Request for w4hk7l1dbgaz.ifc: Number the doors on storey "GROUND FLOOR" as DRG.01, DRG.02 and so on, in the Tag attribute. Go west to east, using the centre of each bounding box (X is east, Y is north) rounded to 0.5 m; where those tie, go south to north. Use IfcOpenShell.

First a look at what the model holds.

```python
import ifcopenshell
import ifcopenshell.util.element
import ifcopenshell.util.placement

model = ifcopenshell.open("w4hk7l1dbgaz.ifc")
print(model.schema)
storey = next(s for s in model.by_type("IfcBuildingStorey") if s.Name == "GROUND FLOOR")
doors = [e for e in ifcopenshell.util.element.get_decomposition(storey) if e.is_a("IfcDoor")]
for e in sorted(doors, key=lambda e: e.id()):
    origin = ifcopenshell.util.placement.get_local_placement(e.ObjectPlacement)[:3, 3]
    print(e.id(), e.Tag, e.Name, origin.round(2) + 0.0, sep=" | ")
```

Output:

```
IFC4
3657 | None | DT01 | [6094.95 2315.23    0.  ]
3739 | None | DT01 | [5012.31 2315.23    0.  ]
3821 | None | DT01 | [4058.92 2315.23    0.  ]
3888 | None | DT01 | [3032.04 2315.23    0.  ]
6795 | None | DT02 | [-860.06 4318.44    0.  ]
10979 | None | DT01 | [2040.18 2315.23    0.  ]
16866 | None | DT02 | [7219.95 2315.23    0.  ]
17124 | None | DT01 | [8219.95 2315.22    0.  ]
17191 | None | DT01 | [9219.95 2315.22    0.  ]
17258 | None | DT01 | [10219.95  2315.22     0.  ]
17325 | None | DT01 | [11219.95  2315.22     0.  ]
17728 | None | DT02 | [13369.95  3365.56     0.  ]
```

```python
import ifcopenshell
import ifcopenshell.geom
import ifcopenshell.util.element
import ifcopenshell.util.shape

model = ifcopenshell.open("w4hk7l1dbgaz.ifc")
settings = ifcopenshell.geom.settings()
settings.set("use-world-coords", True)


def centre(element):
    shape = ifcopenshell.geom.create_shape(settings, element)
    return ifcopenshell.util.shape.get_bbox_centroid(shape.geometry)


storey = next(s for s in model.by_type("IfcBuildingStorey") if s.Name == "GROUND FLOOR")
doors = [e for e in ifcopenshell.util.element.get_decomposition(storey) if e.is_a("IfcDoor")]

# Insertion points can sit at a corner or the storey origin, so sort by the geometry (in metres).
centres = {e: centre(e) for e in doors}
doors.sort(key=lambda e: (round(centres[e][0] / 0.5), centres[e][1]))

for i, e in enumerate(doors, start=1):
    number = f"DRG.{i:02d}"
    e.Tag = number
    print(e.id(), number)

model.write("w4hk7l1dbgaz_v2.ifc")
```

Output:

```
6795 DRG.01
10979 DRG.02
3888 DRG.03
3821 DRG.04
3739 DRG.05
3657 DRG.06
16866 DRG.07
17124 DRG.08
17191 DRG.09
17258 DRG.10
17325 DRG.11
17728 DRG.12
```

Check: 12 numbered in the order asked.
